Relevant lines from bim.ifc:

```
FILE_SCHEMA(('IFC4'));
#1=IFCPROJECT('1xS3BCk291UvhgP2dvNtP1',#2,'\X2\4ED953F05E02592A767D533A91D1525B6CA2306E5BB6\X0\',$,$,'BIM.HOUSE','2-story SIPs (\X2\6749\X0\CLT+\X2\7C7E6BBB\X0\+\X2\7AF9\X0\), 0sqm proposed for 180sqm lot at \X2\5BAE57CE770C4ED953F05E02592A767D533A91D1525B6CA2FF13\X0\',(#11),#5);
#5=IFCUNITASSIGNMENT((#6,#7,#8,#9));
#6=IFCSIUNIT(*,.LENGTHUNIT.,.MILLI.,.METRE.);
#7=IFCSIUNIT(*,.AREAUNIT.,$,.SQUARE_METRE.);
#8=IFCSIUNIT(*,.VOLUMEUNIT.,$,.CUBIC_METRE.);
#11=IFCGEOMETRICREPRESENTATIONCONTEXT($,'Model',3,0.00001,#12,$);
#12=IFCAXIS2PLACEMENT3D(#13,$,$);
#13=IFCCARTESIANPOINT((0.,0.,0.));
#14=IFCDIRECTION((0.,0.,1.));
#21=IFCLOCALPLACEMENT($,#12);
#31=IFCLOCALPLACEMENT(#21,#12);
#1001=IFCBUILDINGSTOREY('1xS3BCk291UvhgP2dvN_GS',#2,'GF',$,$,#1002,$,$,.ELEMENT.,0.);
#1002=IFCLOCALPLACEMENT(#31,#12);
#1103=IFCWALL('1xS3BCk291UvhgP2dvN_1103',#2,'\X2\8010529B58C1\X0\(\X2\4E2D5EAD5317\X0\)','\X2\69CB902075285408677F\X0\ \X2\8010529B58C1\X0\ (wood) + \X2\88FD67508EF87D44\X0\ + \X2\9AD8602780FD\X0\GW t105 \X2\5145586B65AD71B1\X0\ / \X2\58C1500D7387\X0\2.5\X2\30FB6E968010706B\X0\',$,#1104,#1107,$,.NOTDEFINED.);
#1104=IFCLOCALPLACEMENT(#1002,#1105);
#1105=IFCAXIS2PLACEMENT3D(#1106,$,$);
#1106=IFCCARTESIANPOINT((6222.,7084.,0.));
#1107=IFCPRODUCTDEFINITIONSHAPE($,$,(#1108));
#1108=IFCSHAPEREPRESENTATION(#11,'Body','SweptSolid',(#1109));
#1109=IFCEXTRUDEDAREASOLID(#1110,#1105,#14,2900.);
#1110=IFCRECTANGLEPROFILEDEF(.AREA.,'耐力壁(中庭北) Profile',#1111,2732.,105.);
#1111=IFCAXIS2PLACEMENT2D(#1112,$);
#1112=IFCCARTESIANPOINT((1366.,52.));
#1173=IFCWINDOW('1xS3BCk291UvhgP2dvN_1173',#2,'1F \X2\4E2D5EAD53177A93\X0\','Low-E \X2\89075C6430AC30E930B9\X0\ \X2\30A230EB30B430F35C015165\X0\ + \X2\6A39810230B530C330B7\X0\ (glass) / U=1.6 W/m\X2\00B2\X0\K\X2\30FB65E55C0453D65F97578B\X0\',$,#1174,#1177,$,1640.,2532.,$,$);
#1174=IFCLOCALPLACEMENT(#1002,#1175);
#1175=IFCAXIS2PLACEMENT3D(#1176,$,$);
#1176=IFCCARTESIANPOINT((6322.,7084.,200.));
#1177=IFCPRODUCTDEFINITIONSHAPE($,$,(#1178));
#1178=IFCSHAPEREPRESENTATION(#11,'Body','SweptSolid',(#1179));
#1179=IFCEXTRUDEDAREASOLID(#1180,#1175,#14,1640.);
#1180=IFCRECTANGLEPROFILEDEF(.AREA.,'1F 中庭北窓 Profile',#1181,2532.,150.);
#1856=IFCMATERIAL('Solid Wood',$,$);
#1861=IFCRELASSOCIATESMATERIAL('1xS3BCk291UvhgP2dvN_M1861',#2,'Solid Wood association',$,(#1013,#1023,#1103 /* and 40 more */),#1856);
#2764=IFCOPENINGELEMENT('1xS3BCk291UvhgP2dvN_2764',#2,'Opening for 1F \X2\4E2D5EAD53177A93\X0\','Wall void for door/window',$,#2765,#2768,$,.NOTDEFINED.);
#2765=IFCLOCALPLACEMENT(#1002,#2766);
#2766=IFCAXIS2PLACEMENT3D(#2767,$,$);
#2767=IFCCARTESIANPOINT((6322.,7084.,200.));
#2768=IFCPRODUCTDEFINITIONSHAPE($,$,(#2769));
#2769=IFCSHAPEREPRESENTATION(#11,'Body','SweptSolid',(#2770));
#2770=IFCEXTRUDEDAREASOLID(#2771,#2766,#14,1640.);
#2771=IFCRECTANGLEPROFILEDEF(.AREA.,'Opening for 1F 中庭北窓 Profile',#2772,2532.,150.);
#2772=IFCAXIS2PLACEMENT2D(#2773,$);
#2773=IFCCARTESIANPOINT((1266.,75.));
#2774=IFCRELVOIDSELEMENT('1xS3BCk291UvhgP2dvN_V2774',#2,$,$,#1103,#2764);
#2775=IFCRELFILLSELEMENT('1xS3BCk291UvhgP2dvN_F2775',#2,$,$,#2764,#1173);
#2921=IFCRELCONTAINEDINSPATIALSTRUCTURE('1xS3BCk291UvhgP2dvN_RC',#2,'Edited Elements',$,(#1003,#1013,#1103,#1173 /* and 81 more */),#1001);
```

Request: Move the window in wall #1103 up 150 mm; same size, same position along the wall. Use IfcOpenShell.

```python
import numpy as np
import ifcopenshell
import ifcopenshell.api.geometry
import ifcopenshell.util.placement
import ifcopenshell.util.unit

model = ifcopenshell.open("bim.ifc")
unit_scale = ifcopenshell.util.unit.calculate_unit_scale(model)

window = model.by_guid("1xS3BCk291UvhgP2dvN_1173")
opening = window.FillsVoids[0].RelatingOpeningElement
dz = 150.0

shift = np.array([0.0, 0.0, dz])
# The window is not placed relative to its opening, so move both.
for product in (opening, window):
    matrix = ifcopenshell.util.placement.get_local_placement(product.ObjectPlacement)
    matrix[:3, 3] += shift
    ifcopenshell.api.geometry.edit_object_placement(model, product=product, matrix=matrix, is_si=False)

print(f"moved by {dz * unit_scale:+.3f} m")

model.write("bim-out.ifc")
```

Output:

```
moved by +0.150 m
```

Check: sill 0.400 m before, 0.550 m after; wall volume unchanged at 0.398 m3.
